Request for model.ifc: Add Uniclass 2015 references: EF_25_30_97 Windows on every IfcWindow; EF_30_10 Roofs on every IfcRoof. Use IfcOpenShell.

First a look at what the model holds.

```python
import ifcopenshell

model = ifcopenshell.open("model.ifc")
print(model.schema)
print("classifications:", [c.Name for c in model.by_type("IfcClassification")])
for ifc_class in ("IfcDoor", "IfcRoof", "IfcStair", "IfcWall", "IfcWindow"):
    print(ifc_class, len(model.by_type(ifc_class)))
```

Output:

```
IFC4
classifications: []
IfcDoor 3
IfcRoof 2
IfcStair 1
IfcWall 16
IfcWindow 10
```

```python
import ifcopenshell
import ifcopenshell.api.classification

model = ifcopenshell.open("model.ifc")

system = ifcopenshell.api.classification.add_classification(model, classification="Uniclass 2015")

codes = {
    "IfcWindow": ("EF_25_30_97", "Windows"),
    "IfcRoof": ("EF_30_10", "Roofs"),
}
for ifc_class, (code, name) in codes.items():
    products = model.by_type(ifc_class)
    ifcopenshell.api.classification.add_reference(
        model, products=products, classification=system, identification=code, name=name
    )
    print(code, len(products))

model.write("model_v2.ifc")
```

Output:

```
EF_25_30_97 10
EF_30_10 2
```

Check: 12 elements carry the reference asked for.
